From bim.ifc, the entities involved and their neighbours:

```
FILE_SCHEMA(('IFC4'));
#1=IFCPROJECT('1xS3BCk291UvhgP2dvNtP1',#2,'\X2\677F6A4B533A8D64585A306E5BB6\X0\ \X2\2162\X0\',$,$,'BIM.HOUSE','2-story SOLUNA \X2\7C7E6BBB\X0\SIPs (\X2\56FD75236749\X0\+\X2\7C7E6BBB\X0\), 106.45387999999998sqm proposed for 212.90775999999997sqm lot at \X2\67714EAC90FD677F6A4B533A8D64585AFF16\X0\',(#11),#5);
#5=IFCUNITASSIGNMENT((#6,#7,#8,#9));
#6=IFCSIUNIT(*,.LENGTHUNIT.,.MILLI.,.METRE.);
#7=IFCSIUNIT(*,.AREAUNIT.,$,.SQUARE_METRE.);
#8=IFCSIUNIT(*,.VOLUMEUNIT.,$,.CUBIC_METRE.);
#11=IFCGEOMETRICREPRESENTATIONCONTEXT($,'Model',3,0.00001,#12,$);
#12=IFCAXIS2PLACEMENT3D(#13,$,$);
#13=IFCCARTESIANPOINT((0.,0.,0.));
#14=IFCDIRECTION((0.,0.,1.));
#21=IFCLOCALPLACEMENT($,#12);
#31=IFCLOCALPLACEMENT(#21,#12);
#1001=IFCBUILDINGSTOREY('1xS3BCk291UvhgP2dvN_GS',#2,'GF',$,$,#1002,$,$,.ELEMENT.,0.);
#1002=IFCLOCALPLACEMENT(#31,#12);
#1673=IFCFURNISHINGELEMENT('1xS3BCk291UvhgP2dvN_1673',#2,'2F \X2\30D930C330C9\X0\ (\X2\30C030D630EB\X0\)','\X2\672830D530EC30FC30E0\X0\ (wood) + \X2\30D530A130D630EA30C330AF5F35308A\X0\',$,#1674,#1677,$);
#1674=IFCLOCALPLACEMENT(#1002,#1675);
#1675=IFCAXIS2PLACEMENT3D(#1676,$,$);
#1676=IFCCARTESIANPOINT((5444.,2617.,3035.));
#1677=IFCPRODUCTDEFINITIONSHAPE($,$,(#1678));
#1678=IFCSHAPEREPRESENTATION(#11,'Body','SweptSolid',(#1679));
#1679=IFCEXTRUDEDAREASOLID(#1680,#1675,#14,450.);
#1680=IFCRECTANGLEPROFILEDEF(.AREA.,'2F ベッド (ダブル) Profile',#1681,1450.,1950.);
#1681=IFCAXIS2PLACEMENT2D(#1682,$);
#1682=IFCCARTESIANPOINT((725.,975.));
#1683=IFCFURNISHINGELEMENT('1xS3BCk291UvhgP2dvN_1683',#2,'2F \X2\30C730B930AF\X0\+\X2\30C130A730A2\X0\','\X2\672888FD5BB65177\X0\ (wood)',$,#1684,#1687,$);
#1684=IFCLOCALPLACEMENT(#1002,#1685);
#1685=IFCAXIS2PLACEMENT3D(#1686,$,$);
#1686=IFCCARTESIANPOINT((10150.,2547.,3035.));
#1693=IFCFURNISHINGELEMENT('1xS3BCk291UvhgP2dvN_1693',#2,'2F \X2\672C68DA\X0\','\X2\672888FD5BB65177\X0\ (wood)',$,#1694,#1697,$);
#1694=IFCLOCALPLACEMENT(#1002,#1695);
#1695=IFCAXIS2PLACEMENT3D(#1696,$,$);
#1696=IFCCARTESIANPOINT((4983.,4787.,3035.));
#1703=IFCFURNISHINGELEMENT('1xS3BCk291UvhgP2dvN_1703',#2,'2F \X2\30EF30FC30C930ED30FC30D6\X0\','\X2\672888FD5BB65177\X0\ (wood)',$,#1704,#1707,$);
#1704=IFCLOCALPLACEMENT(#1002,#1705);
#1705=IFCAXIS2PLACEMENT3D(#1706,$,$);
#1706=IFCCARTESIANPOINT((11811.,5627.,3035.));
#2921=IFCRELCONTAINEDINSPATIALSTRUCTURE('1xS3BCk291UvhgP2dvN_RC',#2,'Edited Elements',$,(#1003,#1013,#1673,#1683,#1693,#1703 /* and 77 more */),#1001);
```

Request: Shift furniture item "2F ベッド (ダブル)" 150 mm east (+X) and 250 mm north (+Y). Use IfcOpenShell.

```python
import ifcopenshell
import ifcopenshell.api.geometry
import ifcopenshell.util.placement
import ifcopenshell.util.unit

model = ifcopenshell.open("bim.ifc")
unit_scale = ifcopenshell.util.unit.calculate_unit_scale(model)

item = model.by_guid("1xS3BCk291UvhgP2dvN_1673")
matrix = ifcopenshell.util.placement.get_local_placement(item.ObjectPlacement)
matrix[0, 3] += 0.15 / unit_scale
matrix[1, 3] += 0.25 / unit_scale
ifcopenshell.api.geometry.edit_object_placement(model, product=item, matrix=matrix, is_si=False)

print(ifcopenshell.util.placement.get_local_placement(item.ObjectPlacement).round(3) + 0.0)

model.write("bim_v2.ifc")
```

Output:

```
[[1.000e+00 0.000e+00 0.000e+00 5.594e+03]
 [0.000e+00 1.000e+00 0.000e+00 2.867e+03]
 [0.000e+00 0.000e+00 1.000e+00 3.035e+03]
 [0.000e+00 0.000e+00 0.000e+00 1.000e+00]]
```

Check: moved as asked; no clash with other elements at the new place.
